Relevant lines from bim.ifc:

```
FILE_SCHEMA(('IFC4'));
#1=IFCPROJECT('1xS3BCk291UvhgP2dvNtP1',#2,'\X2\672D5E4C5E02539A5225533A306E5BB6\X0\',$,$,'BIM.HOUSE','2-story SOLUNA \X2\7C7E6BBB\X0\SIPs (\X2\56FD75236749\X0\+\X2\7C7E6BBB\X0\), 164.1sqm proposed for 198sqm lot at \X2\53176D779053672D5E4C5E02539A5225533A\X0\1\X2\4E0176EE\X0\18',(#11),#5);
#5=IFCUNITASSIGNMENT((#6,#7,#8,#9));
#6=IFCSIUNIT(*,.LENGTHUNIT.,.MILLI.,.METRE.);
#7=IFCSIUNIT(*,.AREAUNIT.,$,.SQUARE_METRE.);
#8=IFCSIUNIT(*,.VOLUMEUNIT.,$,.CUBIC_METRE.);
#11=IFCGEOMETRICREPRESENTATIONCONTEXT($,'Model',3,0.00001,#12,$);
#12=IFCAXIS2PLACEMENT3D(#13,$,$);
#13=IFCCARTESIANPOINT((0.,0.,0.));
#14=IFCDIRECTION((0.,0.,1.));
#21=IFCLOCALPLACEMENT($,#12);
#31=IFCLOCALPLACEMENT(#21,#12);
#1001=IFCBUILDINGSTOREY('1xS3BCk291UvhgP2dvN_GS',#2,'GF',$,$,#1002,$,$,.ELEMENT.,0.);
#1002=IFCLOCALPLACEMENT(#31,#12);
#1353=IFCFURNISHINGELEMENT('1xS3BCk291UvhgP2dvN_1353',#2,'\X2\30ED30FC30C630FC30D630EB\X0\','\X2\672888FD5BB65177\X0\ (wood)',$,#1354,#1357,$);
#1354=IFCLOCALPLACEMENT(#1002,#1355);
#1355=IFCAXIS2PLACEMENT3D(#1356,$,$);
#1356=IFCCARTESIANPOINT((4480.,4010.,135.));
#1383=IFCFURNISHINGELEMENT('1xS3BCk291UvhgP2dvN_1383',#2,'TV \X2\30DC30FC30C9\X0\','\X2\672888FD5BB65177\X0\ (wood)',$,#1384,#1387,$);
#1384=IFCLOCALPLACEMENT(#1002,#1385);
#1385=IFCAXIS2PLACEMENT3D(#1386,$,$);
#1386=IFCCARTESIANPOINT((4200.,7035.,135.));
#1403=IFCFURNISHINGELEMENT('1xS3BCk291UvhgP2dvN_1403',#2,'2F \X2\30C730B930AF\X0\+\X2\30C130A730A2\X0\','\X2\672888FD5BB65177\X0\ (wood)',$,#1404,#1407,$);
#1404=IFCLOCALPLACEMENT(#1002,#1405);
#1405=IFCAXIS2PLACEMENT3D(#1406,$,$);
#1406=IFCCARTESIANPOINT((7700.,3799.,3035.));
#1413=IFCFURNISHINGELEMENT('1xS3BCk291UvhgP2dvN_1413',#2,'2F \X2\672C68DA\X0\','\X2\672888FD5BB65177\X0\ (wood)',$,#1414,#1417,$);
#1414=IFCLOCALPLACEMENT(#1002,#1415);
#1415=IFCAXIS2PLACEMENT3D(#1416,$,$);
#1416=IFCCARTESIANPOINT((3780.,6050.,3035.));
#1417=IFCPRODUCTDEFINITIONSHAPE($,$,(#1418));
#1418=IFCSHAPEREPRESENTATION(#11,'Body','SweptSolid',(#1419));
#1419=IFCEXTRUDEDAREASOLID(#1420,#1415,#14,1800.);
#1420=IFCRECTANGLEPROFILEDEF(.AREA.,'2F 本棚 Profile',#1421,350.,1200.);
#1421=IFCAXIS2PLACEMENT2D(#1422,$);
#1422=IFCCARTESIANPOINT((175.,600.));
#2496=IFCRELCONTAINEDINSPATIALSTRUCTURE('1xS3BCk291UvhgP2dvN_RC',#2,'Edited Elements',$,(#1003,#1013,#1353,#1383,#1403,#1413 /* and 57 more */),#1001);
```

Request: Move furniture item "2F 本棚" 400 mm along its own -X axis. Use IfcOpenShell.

```python
import ifcopenshell
import ifcopenshell.api.geometry
import ifcopenshell.util.placement
import ifcopenshell.util.unit

model = ifcopenshell.open("bim.ifc")
unit_scale = ifcopenshell.util.unit.calculate_unit_scale(model)

item = model.by_guid("1xS3BCk291UvhgP2dvN_1413")
matrix = ifcopenshell.util.placement.get_local_placement(item.ObjectPlacement)
matrix[:3, 3] -= matrix[:3, 0] * 0.4 / unit_scale
ifcopenshell.api.geometry.edit_object_placement(model, product=item, matrix=matrix, is_si=False)

print(ifcopenshell.util.placement.get_local_placement(item.ObjectPlacement).round(3) + 0.0)

model.write("bim-out.ifc")
```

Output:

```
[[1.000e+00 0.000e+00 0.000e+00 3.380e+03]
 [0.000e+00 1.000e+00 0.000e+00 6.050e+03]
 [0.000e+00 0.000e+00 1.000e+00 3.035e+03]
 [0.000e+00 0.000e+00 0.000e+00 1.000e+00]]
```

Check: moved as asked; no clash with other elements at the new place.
